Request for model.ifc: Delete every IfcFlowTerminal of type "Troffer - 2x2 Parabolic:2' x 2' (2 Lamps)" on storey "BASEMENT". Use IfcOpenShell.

First a look at what the model holds.

```python
import ifcopenshell
import ifcopenshell.util.element

model = ifcopenshell.open("model.ifc")
print(model.schema)
storey = next(s for s in model.by_type("IfcBuildingStorey") if s.Name == "BASEMENT")
terminals = [e for e in ifcopenshell.util.element.get_decomposition(storey) if e.is_a("IfcFlowTerminal")]
seen = {}
for e in terminals:
    element_type = ifcopenshell.util.element.get_type(e)
    name = element_type.Name if element_type not in (None, e) else None
    seen[name] = seen.get(name, 0) + 1
for name, count in sorted(seen.items(), key=str):
    print(count, "x", name)
```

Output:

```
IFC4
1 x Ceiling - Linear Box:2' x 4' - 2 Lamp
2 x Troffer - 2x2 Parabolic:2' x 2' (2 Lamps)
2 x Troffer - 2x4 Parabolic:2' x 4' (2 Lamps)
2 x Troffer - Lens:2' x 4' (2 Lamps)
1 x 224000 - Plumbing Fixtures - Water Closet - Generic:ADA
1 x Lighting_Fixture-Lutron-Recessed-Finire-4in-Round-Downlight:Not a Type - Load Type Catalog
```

```python
import ifcopenshell
import ifcopenshell.api.root
import ifcopenshell.util.element

model = ifcopenshell.open("model.ifc")

storey = next(s for s in model.by_type("IfcBuildingStorey") if s.Name == "BASEMENT")
terminals = [e for e in ifcopenshell.util.element.get_decomposition(storey) if e.is_a("IfcFlowTerminal")]
targets = [e for e in terminals if (t := ifcopenshell.util.element.get_type(e)) not in (None, e) and t.Name == "Troffer - 2x2 Parabolic:2' x 2' (2 Lamps)"]

for e in targets:
    ifcopenshell.api.root.remove_product(model, product=e)
print(len(targets), "removed")

model.write("model-out.ifc")
```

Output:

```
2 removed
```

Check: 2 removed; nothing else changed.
